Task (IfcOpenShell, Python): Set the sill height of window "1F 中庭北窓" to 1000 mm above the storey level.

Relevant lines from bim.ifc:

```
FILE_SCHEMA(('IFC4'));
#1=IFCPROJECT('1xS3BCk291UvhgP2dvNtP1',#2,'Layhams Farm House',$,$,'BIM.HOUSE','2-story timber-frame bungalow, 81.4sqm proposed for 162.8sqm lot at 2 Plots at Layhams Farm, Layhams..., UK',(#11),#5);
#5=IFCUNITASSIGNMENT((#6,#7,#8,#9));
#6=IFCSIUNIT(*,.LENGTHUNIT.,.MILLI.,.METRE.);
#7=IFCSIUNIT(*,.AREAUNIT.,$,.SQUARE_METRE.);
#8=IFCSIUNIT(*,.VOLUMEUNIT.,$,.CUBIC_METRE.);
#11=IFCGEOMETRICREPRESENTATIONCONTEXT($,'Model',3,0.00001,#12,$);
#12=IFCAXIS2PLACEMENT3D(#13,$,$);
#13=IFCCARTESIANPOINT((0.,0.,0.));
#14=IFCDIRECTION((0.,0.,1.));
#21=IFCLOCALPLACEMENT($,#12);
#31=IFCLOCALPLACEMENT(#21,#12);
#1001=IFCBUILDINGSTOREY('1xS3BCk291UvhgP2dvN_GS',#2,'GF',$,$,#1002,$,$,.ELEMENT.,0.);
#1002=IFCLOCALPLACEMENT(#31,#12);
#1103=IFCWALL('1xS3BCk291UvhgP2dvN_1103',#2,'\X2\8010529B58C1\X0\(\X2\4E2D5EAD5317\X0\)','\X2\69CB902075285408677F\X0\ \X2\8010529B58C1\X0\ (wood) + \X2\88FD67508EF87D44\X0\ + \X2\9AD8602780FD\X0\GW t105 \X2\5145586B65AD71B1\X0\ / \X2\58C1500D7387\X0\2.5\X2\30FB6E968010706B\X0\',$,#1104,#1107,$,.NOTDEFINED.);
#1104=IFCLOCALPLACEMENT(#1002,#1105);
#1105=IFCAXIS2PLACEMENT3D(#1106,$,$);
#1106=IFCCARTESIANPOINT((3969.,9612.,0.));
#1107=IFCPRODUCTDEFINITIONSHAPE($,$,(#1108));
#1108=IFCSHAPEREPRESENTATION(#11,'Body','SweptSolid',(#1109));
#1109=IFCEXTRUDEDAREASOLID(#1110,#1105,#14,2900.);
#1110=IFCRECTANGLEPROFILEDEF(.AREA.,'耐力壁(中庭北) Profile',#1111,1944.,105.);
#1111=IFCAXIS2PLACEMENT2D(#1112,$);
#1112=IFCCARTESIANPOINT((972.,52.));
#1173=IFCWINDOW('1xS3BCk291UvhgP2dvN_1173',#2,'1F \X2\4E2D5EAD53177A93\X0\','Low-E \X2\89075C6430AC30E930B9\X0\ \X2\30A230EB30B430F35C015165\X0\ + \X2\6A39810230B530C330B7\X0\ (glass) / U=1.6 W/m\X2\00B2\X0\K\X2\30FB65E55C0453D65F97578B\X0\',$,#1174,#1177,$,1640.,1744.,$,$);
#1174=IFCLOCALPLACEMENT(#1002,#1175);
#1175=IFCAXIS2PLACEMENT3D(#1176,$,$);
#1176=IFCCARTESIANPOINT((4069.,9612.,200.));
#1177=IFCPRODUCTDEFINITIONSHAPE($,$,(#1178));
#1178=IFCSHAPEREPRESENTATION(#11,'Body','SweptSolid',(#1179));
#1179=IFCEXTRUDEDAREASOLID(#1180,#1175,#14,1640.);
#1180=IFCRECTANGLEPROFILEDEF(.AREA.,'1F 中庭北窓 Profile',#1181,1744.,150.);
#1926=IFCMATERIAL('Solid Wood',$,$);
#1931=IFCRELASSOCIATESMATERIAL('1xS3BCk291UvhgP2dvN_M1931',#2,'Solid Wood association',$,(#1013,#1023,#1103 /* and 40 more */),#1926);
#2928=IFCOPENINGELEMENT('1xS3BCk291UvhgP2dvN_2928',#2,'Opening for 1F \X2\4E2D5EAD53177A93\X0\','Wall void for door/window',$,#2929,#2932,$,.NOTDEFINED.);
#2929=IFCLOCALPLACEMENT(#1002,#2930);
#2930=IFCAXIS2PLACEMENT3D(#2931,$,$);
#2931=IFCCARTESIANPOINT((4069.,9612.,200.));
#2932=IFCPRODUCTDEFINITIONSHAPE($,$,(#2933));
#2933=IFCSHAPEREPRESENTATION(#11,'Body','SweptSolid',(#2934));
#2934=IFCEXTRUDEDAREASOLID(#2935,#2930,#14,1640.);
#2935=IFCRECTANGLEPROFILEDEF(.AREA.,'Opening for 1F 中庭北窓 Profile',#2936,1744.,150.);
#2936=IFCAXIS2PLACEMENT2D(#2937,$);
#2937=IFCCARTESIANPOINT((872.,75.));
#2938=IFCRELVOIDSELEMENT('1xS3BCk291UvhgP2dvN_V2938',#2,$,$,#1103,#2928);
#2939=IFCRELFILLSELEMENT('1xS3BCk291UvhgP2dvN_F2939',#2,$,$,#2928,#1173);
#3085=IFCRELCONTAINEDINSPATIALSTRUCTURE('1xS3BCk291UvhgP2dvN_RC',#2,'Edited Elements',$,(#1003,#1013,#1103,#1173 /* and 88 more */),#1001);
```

```python
import numpy as np
import ifcopenshell
import ifcopenshell.api.geometry
import ifcopenshell.geom
import ifcopenshell.util.element
import ifcopenshell.util.placement
import ifcopenshell.util.shape
import ifcopenshell.util.unit

model = ifcopenshell.open("bim.ifc")
unit_scale = ifcopenshell.util.unit.calculate_unit_scale(model)

window = model.by_id(1173)
opening = window.FillsVoids[0].RelatingOpeningElement
storey = ifcopenshell.util.element.get_container(window, ifc_class="IfcBuildingStorey")
level = ifcopenshell.util.placement.get_local_placement(storey.ObjectPlacement)[2, 3]

# The opening's origin need not be at the sill, so measure its lowest point.
shape = ifcopenshell.geom.create_shape(ifcopenshell.geom.settings(), opening)
bottom = ifcopenshell.util.shape.get_shape_bottom_elevation(shape, shape.geometry) / unit_scale
dz = level + 1000.0 - bottom

shift = np.array([0.0, 0.0, dz])
# The window is not placed relative to its opening, so move both.
for product in (opening, window):
    matrix = ifcopenshell.util.placement.get_local_placement(product.ObjectPlacement)
    matrix[:3, 3] += shift
    ifcopenshell.api.geometry.edit_object_placement(model, product=product, matrix=matrix, is_si=False)

print(f"moved by {dz * unit_scale:+.3f} m")

model.write("bim-out.ifc")
```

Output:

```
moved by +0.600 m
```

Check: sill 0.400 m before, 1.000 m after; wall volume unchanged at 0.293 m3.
